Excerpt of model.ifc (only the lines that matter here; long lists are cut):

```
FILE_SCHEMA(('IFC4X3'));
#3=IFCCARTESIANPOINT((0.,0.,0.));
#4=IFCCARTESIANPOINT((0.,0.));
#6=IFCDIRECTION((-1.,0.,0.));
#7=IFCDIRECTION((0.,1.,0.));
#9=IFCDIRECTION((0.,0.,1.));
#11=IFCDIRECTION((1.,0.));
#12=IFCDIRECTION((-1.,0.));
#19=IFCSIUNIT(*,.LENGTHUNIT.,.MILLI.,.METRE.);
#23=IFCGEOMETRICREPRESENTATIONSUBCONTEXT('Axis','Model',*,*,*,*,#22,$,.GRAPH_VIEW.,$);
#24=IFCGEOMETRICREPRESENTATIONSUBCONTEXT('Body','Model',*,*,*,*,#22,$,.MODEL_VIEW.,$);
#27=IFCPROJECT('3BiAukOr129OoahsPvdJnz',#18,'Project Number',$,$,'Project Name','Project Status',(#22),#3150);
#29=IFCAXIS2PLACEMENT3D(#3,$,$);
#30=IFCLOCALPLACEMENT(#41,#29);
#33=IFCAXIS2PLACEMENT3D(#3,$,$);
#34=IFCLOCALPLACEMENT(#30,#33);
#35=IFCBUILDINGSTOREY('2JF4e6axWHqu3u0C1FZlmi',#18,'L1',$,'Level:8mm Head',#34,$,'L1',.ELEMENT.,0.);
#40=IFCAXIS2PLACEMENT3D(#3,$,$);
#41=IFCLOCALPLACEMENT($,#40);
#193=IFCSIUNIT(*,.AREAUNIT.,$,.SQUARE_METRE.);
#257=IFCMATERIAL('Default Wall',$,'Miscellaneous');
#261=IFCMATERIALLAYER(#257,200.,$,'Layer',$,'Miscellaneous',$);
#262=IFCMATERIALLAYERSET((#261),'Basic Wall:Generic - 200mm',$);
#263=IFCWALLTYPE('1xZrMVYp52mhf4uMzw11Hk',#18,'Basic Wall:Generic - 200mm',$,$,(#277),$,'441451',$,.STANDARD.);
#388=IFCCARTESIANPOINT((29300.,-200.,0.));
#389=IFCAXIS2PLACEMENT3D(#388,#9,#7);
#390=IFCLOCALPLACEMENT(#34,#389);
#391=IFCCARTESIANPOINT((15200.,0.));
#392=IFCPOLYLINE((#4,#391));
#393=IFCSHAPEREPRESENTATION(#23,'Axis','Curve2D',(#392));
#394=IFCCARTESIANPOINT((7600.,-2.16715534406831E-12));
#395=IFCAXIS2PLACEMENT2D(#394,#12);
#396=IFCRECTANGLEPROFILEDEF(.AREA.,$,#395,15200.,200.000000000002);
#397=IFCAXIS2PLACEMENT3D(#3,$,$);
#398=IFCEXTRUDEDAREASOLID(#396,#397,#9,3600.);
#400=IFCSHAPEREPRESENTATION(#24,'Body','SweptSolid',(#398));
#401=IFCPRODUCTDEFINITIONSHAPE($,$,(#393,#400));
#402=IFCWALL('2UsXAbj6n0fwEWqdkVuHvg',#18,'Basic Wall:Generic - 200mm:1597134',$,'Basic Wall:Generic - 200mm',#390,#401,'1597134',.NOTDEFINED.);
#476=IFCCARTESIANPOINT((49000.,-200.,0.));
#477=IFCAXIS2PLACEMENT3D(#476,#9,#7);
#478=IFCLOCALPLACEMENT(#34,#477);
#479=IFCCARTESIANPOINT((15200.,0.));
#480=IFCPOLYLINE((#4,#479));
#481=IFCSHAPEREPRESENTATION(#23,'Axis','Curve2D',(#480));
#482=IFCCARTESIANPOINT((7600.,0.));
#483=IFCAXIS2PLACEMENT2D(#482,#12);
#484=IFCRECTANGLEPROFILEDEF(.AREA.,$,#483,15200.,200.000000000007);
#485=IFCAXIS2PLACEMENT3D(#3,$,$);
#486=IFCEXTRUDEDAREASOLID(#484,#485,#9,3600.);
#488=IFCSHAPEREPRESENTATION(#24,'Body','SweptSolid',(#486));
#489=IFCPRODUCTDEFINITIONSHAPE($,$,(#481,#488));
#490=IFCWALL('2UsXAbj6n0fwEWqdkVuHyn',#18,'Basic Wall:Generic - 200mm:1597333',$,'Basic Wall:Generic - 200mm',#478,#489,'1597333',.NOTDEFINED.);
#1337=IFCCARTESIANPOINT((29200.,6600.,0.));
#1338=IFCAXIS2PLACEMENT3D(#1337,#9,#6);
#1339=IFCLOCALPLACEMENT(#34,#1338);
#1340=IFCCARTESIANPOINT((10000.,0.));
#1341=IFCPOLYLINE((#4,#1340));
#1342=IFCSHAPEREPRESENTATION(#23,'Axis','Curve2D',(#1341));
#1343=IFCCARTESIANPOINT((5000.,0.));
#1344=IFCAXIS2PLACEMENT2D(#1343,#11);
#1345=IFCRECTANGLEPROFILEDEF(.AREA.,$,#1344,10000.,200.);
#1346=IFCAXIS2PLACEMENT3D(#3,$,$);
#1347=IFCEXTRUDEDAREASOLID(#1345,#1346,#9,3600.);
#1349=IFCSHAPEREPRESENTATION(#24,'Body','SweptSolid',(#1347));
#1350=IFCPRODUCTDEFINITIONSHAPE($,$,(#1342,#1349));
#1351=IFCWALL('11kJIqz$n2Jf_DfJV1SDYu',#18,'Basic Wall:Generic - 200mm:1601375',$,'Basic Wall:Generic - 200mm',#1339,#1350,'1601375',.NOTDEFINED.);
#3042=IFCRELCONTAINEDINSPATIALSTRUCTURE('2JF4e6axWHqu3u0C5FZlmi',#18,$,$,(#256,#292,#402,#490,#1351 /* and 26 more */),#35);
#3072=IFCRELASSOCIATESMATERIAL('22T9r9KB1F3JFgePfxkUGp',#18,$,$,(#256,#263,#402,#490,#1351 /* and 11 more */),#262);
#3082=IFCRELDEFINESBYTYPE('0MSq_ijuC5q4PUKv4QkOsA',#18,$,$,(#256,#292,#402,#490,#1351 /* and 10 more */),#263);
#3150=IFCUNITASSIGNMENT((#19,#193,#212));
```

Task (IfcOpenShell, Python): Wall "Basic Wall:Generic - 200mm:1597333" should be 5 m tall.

```python
import ifcopenshell
import ifcopenshell.geom
import ifcopenshell.util.representation
import ifcopenshell.util.shape
import ifcopenshell.util.unit

model = ifcopenshell.open("model.ifc")
unit_scale = ifcopenshell.util.unit.calculate_unit_scale(model)
settings = ifcopenshell.geom.settings()


def volume(element):
    """Net volume in cubic metres, openings subtracted."""
    shape = ifcopenshell.geom.create_shape(settings, element)
    return ifcopenshell.util.shape.get_volume(shape.geometry)


wall = model.by_guid("2UsXAbj6n0fwEWqdkVuHyn")
before = volume(wall)

body = ifcopenshell.util.representation.get_representation(wall, "Model", "Body")
solid = body.Items[0]
old_height = solid.Depth
solid.Depth = 5 / unit_scale
after = volume(wall)

print(f"height {old_height:g} -> {solid.Depth:g}, volume {before:.3f} -> {after:.3f} m3")

model.write("model_v2.ifc")
```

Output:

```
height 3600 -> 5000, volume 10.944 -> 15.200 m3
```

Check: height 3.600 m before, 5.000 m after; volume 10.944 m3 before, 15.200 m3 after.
